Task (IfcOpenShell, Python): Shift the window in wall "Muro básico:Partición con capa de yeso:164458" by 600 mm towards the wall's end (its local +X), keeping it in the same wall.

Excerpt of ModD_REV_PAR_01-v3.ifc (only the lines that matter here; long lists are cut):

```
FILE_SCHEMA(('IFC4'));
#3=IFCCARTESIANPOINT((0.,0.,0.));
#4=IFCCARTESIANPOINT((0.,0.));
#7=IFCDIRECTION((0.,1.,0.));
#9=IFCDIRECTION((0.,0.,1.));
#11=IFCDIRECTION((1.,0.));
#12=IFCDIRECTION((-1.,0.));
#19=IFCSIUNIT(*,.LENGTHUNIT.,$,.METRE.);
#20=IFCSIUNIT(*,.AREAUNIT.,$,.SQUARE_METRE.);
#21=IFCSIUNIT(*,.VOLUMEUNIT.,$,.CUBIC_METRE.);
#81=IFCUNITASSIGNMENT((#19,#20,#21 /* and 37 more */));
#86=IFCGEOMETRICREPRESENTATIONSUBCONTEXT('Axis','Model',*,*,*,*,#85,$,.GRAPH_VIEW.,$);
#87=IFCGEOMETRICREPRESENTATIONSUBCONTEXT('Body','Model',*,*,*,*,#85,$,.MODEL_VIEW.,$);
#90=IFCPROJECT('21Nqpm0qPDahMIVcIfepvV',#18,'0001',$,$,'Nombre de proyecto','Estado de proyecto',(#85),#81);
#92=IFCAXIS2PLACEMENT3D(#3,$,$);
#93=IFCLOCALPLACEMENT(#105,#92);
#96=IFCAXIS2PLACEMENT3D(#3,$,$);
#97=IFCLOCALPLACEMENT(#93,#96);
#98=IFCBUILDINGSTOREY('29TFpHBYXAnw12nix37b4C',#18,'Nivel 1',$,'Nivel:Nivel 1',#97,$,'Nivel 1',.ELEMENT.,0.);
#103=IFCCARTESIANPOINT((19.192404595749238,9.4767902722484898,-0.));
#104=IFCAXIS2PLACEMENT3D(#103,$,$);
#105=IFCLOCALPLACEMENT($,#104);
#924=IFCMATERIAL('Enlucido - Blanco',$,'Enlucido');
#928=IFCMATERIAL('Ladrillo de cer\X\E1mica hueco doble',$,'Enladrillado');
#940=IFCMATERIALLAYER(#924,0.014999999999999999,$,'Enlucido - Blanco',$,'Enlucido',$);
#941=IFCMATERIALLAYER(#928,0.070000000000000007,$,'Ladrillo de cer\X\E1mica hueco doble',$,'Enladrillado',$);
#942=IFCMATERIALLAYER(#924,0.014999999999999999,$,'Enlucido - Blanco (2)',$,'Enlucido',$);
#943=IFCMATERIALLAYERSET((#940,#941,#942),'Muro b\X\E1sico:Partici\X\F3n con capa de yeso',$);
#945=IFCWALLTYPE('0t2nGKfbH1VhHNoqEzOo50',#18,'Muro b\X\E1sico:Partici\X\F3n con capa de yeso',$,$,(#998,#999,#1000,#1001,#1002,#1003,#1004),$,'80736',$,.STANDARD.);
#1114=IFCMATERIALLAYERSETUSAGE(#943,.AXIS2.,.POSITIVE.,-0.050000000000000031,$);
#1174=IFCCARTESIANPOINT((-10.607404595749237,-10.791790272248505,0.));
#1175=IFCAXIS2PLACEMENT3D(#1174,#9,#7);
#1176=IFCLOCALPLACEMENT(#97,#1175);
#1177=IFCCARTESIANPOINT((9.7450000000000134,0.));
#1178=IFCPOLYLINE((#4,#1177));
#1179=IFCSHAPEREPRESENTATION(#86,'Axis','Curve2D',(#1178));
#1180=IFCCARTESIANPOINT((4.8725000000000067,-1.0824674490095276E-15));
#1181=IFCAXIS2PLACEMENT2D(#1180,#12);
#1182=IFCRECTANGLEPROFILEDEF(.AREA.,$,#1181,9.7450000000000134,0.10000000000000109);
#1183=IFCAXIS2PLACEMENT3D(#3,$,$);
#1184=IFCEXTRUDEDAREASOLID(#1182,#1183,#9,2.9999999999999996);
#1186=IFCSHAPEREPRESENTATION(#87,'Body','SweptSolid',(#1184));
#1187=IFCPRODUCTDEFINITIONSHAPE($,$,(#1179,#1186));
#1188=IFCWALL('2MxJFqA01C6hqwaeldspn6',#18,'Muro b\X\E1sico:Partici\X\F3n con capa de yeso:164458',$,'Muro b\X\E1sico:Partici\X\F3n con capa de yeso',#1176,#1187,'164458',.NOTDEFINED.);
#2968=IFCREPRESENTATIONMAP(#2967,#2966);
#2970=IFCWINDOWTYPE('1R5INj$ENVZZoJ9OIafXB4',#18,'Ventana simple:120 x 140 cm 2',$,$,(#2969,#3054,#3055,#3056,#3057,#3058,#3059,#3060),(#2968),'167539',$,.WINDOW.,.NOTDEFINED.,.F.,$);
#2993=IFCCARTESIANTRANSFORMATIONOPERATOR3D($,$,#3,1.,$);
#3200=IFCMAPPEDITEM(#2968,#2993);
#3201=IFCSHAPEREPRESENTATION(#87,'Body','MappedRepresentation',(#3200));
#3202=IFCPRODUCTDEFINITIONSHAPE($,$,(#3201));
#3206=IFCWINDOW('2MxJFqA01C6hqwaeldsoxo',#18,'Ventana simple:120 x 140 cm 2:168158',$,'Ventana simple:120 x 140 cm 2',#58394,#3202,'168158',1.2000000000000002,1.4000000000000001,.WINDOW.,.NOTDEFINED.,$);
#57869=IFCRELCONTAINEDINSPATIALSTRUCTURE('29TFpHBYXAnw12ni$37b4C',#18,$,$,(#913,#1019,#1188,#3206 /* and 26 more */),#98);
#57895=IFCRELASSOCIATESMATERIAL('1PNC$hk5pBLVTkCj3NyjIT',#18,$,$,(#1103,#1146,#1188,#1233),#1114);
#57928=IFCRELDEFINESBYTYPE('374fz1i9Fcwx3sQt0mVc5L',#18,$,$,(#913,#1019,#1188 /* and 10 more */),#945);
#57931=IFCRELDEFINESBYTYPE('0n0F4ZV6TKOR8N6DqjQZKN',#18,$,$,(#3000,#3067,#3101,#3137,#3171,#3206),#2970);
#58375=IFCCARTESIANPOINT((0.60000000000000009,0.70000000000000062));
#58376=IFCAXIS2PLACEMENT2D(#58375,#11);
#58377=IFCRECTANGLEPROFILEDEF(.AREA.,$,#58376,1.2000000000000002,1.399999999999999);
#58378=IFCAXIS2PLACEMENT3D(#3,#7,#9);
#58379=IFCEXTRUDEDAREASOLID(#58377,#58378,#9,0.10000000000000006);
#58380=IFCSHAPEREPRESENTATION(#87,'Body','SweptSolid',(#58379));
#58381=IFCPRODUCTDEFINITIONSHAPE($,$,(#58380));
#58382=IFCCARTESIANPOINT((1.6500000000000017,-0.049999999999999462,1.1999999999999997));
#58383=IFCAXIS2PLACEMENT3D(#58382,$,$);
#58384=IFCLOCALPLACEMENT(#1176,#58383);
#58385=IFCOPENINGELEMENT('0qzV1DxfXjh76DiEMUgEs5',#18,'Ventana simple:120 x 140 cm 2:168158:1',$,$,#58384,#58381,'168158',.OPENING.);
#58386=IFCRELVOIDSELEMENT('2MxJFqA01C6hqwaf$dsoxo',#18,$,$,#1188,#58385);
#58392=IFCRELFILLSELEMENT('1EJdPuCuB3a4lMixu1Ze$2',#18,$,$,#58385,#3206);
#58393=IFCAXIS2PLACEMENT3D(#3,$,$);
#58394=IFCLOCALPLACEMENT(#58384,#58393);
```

```python
import ifcopenshell
import ifcopenshell.api.geometry
import ifcopenshell.util.placement
import ifcopenshell.util.unit

model = ifcopenshell.open("ModD_REV_PAR_01-v3.ifc")
unit_scale = ifcopenshell.util.unit.calculate_unit_scale(model)

window = model.by_guid("2MxJFqA01C6hqwaeldsoxo")
opening = window.FillsVoids[0].RelatingOpeningElement
wall = opening.VoidsElements[0].RelatingBuildingElement

wall_matrix = ifcopenshell.util.placement.get_local_placement(wall.ObjectPlacement)
shift = wall_matrix[:3, 0] * 0.6 / unit_scale
before = ifcopenshell.util.placement.get_local_placement(window.ObjectPlacement)[:3, 3].copy()

# The window is placed relative to its opening, so it follows when the opening moves.
matrix = ifcopenshell.util.placement.get_local_placement(opening.ObjectPlacement)
matrix[:3, 3] += shift
ifcopenshell.api.geometry.edit_object_placement(
    model, product=opening, matrix=matrix, is_si=False, should_transform_children=True
)

after = ifcopenshell.util.placement.get_local_placement(window.ObjectPlacement)[:3, 3]
print("window moved by", (after - before).round(3) + 0.0)

model.write("ModD_REV_PAR_01-v3_updated.ifc")
```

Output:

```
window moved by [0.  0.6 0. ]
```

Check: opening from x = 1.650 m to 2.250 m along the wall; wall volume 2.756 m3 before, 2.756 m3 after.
